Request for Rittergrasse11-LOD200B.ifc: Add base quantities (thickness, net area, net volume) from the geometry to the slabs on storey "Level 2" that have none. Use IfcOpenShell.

First a look at what the model holds.

```python
import ifcopenshell
import ifcopenshell.util.element
import ifcopenshell.util.unit

model = ifcopenshell.open("Rittergrasse11-LOD200B.ifc")
print(model.schema)
for unit_type in ("LENGTHUNIT", "AREAUNIT", "VOLUMEUNIT"):
    print(unit_type, ifcopenshell.util.unit.calculate_unit_scale(model, unit_type))
storey = next(s for s in model.by_type("IfcBuildingStorey") if s.Name == "Level 2")
slabs = [e for e in ifcopenshell.util.element.get_decomposition(storey) if e.is_a("IfcSlab")]
for e in sorted(slabs, key=lambda e: e.id()):
    print(e.id(), e.is_a(), e.Name, list(ifcopenshell.util.element.get_psets(e, qtos_only=True)), sep=" | ")
```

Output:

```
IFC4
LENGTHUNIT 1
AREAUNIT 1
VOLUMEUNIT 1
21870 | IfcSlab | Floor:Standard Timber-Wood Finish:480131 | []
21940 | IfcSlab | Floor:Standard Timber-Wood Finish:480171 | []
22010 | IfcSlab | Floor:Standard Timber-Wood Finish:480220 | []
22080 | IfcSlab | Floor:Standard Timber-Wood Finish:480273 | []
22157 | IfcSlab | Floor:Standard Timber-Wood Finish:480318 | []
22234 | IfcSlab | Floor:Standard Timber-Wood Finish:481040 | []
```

```python
import ifcopenshell
import ifcopenshell.api.pset
import ifcopenshell.geom
import ifcopenshell.util.element
import ifcopenshell.util.shape
import ifcopenshell.util.unit

model = ifcopenshell.open("Rittergrasse11-LOD200B.ifc")
unit_scale = ifcopenshell.util.unit.calculate_unit_scale(model)
area_scale = ifcopenshell.util.unit.calculate_unit_scale(model, "AREAUNIT")
volume_scale = ifcopenshell.util.unit.calculate_unit_scale(model, "VOLUMEUNIT")
settings = ifcopenshell.geom.settings()

storey = next(s for s in model.by_type("IfcBuildingStorey") if s.Name == "Level 2")
slabs = [e for e in ifcopenshell.util.element.get_decomposition(storey) if e.is_a("IfcSlab")]

for e in sorted(slabs, key=lambda e: e.id()):
    if ifcopenshell.util.element.get_psets(e, qtos_only=True, should_inherit=False):
        continue
    # Geometry comes back in metres, in the element's own axes.
    shape = ifcopenshell.geom.create_shape(settings, e)
    values = {
        "Width": ifcopenshell.util.shape.get_z(shape.geometry) / unit_scale,
        "NetArea": ifcopenshell.util.shape.get_footprint_area(shape.geometry) / area_scale,
        "NetVolume": ifcopenshell.util.shape.get_volume(shape.geometry) / volume_scale,
    }
    qto = ifcopenshell.api.pset.add_qto(model, product=e, name="Qto_SlabBaseQuantities")
    ifcopenshell.api.pset.edit_qto(model, qto=qto, properties=values)
    print(e.id(), {k: round(v, 3) for k, v in values.items()})

model.write("Rittergrasse11-LOD200B_v2.ifc")
```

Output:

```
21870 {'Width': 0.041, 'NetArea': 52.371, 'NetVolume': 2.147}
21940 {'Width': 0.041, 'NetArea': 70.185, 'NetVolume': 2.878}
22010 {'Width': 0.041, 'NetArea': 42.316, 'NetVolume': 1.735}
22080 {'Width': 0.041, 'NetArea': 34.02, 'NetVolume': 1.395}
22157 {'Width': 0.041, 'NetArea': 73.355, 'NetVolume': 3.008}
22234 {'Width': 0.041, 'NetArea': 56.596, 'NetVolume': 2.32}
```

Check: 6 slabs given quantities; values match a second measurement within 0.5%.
